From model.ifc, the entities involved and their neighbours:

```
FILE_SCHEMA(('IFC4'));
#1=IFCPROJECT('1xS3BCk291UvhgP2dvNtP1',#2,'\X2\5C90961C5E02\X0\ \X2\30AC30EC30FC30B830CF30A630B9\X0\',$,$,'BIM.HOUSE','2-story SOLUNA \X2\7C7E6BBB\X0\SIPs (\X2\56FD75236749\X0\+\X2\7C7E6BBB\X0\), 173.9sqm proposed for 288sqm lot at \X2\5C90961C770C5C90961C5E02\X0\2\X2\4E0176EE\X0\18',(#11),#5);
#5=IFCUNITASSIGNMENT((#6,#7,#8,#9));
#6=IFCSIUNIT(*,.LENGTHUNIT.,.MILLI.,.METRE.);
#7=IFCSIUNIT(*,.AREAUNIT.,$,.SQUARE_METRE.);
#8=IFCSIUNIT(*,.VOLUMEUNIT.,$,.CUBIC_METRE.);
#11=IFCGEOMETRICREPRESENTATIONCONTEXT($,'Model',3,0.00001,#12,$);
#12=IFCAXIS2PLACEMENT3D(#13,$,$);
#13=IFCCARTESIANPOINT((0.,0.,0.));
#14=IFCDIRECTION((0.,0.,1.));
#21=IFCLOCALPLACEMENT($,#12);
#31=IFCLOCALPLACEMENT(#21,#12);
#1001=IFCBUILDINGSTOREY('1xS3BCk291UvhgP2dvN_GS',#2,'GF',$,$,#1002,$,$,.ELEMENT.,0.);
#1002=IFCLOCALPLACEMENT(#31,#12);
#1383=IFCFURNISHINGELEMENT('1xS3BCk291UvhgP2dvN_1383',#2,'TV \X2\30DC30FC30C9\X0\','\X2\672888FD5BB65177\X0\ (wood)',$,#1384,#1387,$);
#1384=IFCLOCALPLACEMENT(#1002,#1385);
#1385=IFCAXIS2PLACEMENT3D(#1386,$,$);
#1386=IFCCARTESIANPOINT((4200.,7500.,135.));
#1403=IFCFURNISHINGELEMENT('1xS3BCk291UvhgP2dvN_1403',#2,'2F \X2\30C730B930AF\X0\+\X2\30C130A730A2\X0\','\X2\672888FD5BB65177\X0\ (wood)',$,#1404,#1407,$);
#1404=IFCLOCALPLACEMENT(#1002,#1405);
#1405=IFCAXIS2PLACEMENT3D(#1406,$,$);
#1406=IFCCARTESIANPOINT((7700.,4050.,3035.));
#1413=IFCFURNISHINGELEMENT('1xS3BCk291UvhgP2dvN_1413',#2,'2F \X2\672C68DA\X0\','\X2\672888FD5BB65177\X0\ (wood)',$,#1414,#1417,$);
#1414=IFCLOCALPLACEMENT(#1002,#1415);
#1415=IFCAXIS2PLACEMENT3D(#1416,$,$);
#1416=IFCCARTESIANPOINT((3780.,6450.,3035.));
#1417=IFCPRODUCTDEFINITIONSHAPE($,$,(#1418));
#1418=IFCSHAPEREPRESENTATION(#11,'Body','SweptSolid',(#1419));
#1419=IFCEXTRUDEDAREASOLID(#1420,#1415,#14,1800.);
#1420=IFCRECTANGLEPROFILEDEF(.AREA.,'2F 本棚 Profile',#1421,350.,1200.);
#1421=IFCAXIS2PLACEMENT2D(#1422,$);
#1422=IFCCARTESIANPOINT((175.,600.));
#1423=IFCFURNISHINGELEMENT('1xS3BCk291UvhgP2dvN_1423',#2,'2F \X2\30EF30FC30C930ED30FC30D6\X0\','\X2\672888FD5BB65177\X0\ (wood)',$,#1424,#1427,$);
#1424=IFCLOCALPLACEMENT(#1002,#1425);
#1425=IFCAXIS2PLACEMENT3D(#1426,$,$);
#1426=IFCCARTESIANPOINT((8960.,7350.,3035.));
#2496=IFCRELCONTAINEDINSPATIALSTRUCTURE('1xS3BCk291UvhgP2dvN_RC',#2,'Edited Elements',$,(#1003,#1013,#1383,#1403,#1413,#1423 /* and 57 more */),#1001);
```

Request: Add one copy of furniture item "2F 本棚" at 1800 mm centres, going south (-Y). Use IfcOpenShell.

```python
import numpy as np
import ifcopenshell
import ifcopenshell.api.geometry
import ifcopenshell.api.root
import ifcopenshell.util.element
import ifcopenshell.util.placement
import ifcopenshell.util.unit

model = ifcopenshell.open("model.ifc")
unit_scale = ifcopenshell.util.unit.calculate_unit_scale(model)


def reuse_history(source, copy):
    """copy_class also copies each property set's owner history, people and application; keep the originals."""
    for rel in copy.IsDefinedBy:
        if rel.is_a("IfcRelDefinesByProperties") and (history := rel.RelatingPropertyDefinition.OwnerHistory):
            rel.RelatingPropertyDefinition.OwnerHistory = source.OwnerHistory
            ifcopenshell.util.element.remove_deep2(model, history)


source = model.by_guid("1xS3BCk291UvhgP2dvN_1413")
base = ifcopenshell.util.placement.get_local_placement(source.ObjectPlacement)
step = np.array([0.0, -1.0, 0.0]) * 1.8 / unit_scale

for i in range(1, 2):
    copy = ifcopenshell.api.root.copy_class(model, product=source)
    copy.Representation = ifcopenshell.util.element.copy_deep(
        model, source.Representation, exclude=["IfcGeometricRepresentationContext", "IfcRepresentationMap"]
    )
    reuse_history(source, copy)
    matrix = base.copy()
    matrix[:3, 3] += i * step
    print("added at", matrix[:3, 3].round(3) + 0.0)
    ifcopenshell.api.geometry.edit_object_placement(model, product=copy, matrix=matrix, is_si=False)

model.write("model_rev.ifc")
```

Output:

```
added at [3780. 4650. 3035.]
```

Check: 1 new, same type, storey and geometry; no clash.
